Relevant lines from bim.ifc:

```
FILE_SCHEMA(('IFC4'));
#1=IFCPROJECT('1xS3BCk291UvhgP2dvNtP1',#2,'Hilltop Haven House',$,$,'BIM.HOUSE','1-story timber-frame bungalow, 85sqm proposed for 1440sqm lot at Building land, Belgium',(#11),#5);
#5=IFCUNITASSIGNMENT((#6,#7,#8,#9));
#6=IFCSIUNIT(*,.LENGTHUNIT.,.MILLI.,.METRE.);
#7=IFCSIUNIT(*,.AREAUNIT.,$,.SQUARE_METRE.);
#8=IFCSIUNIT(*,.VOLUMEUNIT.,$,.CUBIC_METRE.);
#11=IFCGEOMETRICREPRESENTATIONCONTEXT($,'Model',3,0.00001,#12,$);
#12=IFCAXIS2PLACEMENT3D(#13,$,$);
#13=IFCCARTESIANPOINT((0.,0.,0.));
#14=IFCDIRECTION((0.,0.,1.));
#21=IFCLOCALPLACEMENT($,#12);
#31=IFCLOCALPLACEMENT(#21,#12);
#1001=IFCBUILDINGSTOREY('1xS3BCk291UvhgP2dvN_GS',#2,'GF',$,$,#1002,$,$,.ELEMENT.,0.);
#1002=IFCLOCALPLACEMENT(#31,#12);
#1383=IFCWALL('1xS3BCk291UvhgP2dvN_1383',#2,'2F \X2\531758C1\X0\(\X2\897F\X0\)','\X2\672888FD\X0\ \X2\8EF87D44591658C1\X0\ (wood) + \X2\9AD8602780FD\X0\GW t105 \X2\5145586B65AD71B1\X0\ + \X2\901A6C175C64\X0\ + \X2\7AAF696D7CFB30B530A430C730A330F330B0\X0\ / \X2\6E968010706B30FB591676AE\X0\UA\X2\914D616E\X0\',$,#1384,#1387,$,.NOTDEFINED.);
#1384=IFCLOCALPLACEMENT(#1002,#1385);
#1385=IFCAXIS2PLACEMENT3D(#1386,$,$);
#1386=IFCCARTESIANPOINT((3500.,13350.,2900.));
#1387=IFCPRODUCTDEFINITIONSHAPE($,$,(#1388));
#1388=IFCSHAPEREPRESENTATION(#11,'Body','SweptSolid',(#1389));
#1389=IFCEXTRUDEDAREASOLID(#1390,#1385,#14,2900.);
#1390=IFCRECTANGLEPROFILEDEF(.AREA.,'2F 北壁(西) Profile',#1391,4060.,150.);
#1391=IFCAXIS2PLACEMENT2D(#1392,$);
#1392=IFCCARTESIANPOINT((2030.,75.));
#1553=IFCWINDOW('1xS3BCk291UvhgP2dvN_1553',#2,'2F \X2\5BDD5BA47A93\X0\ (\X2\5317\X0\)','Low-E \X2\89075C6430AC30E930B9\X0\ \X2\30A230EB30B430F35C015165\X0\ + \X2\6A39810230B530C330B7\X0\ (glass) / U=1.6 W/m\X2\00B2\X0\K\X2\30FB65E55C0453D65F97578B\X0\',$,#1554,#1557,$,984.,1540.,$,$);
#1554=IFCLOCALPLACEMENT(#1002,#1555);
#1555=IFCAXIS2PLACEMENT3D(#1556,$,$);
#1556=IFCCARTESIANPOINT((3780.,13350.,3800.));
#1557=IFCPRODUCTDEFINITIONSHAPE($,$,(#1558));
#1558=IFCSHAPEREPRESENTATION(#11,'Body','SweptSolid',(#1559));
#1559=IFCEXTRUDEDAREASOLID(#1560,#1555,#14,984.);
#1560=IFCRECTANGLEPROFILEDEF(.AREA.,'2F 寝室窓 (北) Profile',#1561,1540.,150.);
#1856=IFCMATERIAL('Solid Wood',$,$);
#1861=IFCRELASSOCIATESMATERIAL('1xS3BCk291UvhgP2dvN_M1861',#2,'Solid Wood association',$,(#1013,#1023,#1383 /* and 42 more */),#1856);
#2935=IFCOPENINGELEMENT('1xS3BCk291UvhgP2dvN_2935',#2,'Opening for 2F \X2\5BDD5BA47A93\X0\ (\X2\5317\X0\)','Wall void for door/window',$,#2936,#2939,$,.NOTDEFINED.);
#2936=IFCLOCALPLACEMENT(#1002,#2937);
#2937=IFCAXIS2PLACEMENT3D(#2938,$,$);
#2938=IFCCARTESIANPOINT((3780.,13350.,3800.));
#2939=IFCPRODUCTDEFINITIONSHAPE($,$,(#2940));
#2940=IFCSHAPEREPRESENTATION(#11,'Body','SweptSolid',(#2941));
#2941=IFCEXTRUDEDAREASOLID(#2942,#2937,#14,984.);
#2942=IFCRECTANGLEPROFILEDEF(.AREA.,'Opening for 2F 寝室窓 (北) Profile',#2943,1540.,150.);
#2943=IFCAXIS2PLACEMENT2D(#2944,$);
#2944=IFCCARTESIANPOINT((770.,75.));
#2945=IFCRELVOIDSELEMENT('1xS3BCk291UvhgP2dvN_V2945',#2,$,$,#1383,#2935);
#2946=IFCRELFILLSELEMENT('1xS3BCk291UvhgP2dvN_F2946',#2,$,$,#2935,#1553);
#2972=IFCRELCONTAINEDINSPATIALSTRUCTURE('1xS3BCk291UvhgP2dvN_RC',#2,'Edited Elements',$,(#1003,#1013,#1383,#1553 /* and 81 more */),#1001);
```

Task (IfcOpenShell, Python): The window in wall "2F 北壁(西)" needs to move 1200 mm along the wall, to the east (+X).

```python
import ifcopenshell
import ifcopenshell.api.geometry
import ifcopenshell.util.placement

model = ifcopenshell.open("bim.ifc")

window = model.by_id(1553)
opening = window.FillsVoids[0].RelatingOpeningElement
wall = opening.VoidsElements[0].RelatingBuildingElement

wall_matrix = ifcopenshell.util.placement.get_local_placement(wall.ObjectPlacement)
shift = wall_matrix[:3, 0] * 1200.0
before = ifcopenshell.util.placement.get_local_placement(window.ObjectPlacement)[:3, 3].copy()

# The window is not placed relative to its opening, so move both.
for product in (opening, window):
    matrix = ifcopenshell.util.placement.get_local_placement(product.ObjectPlacement)
    matrix[:3, 3] += shift
    ifcopenshell.api.geometry.edit_object_placement(model, product=product, matrix=matrix, is_si=False)

after = ifcopenshell.util.placement.get_local_placement(window.ObjectPlacement)[:3, 3]
print("window moved by", (after - before).round(3) + 0.0)

model.write("bim_updated.ifc")
```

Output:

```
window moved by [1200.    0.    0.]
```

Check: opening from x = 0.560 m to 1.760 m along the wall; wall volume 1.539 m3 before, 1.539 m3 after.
